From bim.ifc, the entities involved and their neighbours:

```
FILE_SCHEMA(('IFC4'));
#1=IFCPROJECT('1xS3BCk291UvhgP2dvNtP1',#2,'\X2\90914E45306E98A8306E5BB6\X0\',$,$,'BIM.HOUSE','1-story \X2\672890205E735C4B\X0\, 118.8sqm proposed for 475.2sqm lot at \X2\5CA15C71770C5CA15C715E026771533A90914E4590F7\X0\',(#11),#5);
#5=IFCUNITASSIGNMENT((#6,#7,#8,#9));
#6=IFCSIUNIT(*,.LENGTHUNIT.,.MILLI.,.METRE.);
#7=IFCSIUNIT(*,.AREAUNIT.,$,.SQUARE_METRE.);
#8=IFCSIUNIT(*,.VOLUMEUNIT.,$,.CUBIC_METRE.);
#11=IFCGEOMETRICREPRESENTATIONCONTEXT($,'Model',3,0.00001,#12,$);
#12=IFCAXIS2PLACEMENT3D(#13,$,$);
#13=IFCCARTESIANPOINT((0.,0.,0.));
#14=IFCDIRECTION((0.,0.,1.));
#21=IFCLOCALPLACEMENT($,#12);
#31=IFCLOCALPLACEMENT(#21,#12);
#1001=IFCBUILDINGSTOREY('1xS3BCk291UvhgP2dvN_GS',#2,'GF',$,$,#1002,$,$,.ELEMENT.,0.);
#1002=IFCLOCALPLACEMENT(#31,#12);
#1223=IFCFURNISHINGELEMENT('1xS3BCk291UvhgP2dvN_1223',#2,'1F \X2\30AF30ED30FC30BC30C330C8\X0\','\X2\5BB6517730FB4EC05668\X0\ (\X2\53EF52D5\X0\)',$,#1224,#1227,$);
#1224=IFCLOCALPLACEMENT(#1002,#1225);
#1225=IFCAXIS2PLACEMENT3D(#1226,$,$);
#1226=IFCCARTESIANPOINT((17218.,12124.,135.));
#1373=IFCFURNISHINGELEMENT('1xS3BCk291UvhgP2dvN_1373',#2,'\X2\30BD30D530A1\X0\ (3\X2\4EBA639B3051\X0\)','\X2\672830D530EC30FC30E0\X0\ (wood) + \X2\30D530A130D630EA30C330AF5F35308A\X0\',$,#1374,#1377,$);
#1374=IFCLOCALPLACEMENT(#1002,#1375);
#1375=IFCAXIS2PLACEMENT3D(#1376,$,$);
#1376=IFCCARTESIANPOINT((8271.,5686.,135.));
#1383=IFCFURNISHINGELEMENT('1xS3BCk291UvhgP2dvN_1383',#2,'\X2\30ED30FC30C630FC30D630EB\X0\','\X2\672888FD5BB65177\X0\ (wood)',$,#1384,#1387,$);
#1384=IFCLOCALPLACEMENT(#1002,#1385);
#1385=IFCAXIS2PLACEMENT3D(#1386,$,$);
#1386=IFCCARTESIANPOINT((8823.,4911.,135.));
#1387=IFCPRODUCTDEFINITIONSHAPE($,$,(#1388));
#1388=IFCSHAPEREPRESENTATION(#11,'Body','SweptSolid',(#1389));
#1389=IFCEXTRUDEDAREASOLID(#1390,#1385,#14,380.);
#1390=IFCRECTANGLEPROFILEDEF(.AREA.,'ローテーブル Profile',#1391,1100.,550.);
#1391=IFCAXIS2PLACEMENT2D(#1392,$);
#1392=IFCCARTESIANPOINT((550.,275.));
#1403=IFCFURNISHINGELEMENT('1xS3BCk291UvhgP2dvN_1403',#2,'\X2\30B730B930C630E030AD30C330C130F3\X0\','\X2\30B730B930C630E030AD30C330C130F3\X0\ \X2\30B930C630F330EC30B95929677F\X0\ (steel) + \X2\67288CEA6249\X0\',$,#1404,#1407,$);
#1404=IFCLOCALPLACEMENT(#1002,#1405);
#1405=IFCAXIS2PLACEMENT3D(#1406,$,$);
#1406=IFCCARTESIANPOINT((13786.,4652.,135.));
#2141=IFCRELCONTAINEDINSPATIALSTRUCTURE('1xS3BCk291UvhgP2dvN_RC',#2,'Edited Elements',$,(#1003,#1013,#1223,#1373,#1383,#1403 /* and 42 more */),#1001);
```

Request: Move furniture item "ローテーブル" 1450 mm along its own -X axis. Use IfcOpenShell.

```python
import ifcopenshell
import ifcopenshell.api.geometry
import ifcopenshell.util.placement

model = ifcopenshell.open("bim.ifc")

item = model.by_guid("1xS3BCk291UvhgP2dvN_1383")
matrix = ifcopenshell.util.placement.get_local_placement(item.ObjectPlacement)
matrix[:3, 3] -= matrix[:3, 0] * 1450.0
ifcopenshell.api.geometry.edit_object_placement(model, product=item, matrix=matrix, is_si=False)

print(ifcopenshell.util.placement.get_local_placement(item.ObjectPlacement).round(3) + 0.0)

model.write("bim_updated.ifc")
```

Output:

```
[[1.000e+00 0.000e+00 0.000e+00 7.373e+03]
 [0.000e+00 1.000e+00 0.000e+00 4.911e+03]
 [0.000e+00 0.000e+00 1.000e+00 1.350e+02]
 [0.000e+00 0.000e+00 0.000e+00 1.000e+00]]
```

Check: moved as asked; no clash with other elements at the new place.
